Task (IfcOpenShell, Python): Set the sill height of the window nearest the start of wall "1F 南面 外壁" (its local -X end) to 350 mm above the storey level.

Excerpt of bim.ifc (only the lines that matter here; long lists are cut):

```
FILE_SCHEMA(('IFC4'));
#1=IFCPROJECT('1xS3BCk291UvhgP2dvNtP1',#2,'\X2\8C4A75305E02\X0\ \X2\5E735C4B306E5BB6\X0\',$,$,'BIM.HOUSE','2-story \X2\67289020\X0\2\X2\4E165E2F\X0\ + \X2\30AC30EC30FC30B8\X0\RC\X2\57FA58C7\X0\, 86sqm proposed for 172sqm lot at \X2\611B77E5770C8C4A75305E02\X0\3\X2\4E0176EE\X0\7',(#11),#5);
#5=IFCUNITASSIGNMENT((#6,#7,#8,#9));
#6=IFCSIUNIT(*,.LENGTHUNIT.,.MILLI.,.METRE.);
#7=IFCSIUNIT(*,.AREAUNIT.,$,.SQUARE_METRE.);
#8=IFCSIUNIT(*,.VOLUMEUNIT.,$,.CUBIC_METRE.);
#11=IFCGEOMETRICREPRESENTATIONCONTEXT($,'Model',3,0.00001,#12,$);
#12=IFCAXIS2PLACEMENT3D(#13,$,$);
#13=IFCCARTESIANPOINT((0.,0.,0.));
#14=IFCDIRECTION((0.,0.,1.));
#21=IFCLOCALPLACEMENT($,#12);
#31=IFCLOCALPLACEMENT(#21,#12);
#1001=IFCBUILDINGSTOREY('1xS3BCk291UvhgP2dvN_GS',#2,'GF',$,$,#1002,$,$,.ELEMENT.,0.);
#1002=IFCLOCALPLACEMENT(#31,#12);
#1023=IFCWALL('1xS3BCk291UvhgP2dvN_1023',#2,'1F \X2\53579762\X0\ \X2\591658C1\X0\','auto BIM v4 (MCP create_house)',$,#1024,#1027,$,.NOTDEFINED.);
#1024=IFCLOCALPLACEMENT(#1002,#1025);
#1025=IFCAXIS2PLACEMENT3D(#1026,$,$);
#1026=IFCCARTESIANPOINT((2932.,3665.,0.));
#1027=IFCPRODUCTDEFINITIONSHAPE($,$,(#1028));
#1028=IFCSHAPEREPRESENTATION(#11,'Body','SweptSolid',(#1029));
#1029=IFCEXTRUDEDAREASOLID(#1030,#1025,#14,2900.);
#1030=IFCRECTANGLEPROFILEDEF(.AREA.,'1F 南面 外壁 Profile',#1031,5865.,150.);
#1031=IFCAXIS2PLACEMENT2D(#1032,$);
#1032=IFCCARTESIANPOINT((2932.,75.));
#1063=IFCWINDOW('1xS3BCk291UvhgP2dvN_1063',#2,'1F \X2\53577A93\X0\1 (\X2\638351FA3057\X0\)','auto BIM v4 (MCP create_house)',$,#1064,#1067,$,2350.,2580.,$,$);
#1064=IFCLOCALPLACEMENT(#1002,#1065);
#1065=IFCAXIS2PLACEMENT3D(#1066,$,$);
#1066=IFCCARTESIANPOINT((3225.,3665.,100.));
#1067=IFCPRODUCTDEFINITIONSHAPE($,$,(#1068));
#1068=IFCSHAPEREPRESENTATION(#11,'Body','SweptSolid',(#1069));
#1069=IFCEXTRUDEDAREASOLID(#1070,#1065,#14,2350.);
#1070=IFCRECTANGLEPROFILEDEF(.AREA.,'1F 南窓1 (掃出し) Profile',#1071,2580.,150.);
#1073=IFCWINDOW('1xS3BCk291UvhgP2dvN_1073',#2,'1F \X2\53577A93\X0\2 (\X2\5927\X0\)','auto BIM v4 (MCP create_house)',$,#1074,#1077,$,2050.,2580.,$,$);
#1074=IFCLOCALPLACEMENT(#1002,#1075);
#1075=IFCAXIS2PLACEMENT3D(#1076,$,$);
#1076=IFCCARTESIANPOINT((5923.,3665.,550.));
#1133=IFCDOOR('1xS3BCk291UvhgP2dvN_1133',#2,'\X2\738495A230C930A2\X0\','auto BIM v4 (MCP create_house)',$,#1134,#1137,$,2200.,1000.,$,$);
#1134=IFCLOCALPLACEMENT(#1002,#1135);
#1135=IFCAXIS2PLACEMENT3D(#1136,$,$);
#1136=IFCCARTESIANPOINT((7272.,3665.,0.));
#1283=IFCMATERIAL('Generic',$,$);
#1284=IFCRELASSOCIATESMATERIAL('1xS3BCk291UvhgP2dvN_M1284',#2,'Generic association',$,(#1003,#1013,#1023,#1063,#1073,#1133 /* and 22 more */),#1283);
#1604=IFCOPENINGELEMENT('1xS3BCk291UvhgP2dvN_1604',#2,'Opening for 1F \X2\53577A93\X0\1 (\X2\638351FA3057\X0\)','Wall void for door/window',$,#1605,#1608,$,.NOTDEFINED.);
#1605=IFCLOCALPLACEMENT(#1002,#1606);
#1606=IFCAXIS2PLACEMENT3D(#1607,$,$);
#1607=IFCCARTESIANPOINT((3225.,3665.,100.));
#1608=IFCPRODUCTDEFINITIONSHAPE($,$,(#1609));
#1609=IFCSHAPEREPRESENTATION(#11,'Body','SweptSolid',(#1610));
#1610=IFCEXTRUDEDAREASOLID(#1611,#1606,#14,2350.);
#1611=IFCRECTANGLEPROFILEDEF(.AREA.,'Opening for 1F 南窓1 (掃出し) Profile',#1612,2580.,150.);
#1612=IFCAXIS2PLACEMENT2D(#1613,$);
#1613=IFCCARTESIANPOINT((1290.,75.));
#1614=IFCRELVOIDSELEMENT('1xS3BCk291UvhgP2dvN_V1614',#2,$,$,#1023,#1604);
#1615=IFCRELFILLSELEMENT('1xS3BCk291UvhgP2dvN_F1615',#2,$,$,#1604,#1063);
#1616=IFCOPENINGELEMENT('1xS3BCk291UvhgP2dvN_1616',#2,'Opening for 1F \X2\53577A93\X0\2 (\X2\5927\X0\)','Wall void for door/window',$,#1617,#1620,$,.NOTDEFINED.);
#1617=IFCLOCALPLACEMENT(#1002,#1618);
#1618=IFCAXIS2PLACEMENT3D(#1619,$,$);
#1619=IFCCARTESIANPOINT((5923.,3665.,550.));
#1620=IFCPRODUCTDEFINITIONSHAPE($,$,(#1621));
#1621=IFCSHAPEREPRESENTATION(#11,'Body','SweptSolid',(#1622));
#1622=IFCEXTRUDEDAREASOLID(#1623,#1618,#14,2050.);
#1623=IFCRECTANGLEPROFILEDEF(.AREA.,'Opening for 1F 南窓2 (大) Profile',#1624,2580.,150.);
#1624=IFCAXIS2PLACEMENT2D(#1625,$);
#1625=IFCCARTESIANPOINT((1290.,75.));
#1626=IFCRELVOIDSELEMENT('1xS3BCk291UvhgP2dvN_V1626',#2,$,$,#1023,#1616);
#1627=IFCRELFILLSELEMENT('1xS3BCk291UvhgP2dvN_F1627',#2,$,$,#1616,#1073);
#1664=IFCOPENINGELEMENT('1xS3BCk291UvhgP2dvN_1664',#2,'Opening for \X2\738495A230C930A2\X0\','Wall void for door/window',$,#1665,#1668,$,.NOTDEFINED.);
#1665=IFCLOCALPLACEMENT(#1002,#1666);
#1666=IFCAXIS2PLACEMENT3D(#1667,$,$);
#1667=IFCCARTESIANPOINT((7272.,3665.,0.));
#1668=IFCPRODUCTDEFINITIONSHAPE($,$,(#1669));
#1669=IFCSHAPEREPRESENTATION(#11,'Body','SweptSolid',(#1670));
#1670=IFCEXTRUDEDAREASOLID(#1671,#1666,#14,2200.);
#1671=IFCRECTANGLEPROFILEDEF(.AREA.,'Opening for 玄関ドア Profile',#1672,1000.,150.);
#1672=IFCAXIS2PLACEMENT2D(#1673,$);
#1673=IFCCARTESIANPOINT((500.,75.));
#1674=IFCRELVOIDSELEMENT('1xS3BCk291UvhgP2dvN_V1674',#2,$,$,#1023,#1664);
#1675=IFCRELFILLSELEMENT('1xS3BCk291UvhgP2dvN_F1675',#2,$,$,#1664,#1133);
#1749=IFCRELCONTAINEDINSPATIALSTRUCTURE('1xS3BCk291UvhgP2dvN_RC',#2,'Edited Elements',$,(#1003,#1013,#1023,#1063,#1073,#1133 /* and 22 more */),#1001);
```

```python
import numpy as np
import ifcopenshell
import ifcopenshell.api.geometry
import ifcopenshell.geom
import ifcopenshell.util.element
import ifcopenshell.util.placement
import ifcopenshell.util.shape
import ifcopenshell.util.unit

model = ifcopenshell.open("bim.ifc")
unit_scale = ifcopenshell.util.unit.calculate_unit_scale(model)

window = model.by_guid("1xS3BCk291UvhgP2dvN_1063")
opening = window.FillsVoids[0].RelatingOpeningElement
storey = ifcopenshell.util.element.get_container(window, ifc_class="IfcBuildingStorey")
level = ifcopenshell.util.placement.get_local_placement(storey.ObjectPlacement)[2, 3]

# The opening's origin need not be at the sill, so measure its lowest point.
shape = ifcopenshell.geom.create_shape(ifcopenshell.geom.settings(), opening)
bottom = ifcopenshell.util.shape.get_shape_bottom_elevation(shape, shape.geometry) / unit_scale
dz = level + 0.35 / unit_scale - bottom

shift = np.array([0.0, 0.0, dz])
# The window is not placed relative to its opening, so move both.
for product in (opening, window):
    matrix = ifcopenshell.util.placement.get_local_placement(product.ObjectPlacement)
    matrix[:3, 3] += shift
    ifcopenshell.api.geometry.edit_object_placement(model, product=product, matrix=matrix, is_si=False)

print(f"moved by {dz * unit_scale:+.3f} m")

model.write("bim_rev.ifc")
```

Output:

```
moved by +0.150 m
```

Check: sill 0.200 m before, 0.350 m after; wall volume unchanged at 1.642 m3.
